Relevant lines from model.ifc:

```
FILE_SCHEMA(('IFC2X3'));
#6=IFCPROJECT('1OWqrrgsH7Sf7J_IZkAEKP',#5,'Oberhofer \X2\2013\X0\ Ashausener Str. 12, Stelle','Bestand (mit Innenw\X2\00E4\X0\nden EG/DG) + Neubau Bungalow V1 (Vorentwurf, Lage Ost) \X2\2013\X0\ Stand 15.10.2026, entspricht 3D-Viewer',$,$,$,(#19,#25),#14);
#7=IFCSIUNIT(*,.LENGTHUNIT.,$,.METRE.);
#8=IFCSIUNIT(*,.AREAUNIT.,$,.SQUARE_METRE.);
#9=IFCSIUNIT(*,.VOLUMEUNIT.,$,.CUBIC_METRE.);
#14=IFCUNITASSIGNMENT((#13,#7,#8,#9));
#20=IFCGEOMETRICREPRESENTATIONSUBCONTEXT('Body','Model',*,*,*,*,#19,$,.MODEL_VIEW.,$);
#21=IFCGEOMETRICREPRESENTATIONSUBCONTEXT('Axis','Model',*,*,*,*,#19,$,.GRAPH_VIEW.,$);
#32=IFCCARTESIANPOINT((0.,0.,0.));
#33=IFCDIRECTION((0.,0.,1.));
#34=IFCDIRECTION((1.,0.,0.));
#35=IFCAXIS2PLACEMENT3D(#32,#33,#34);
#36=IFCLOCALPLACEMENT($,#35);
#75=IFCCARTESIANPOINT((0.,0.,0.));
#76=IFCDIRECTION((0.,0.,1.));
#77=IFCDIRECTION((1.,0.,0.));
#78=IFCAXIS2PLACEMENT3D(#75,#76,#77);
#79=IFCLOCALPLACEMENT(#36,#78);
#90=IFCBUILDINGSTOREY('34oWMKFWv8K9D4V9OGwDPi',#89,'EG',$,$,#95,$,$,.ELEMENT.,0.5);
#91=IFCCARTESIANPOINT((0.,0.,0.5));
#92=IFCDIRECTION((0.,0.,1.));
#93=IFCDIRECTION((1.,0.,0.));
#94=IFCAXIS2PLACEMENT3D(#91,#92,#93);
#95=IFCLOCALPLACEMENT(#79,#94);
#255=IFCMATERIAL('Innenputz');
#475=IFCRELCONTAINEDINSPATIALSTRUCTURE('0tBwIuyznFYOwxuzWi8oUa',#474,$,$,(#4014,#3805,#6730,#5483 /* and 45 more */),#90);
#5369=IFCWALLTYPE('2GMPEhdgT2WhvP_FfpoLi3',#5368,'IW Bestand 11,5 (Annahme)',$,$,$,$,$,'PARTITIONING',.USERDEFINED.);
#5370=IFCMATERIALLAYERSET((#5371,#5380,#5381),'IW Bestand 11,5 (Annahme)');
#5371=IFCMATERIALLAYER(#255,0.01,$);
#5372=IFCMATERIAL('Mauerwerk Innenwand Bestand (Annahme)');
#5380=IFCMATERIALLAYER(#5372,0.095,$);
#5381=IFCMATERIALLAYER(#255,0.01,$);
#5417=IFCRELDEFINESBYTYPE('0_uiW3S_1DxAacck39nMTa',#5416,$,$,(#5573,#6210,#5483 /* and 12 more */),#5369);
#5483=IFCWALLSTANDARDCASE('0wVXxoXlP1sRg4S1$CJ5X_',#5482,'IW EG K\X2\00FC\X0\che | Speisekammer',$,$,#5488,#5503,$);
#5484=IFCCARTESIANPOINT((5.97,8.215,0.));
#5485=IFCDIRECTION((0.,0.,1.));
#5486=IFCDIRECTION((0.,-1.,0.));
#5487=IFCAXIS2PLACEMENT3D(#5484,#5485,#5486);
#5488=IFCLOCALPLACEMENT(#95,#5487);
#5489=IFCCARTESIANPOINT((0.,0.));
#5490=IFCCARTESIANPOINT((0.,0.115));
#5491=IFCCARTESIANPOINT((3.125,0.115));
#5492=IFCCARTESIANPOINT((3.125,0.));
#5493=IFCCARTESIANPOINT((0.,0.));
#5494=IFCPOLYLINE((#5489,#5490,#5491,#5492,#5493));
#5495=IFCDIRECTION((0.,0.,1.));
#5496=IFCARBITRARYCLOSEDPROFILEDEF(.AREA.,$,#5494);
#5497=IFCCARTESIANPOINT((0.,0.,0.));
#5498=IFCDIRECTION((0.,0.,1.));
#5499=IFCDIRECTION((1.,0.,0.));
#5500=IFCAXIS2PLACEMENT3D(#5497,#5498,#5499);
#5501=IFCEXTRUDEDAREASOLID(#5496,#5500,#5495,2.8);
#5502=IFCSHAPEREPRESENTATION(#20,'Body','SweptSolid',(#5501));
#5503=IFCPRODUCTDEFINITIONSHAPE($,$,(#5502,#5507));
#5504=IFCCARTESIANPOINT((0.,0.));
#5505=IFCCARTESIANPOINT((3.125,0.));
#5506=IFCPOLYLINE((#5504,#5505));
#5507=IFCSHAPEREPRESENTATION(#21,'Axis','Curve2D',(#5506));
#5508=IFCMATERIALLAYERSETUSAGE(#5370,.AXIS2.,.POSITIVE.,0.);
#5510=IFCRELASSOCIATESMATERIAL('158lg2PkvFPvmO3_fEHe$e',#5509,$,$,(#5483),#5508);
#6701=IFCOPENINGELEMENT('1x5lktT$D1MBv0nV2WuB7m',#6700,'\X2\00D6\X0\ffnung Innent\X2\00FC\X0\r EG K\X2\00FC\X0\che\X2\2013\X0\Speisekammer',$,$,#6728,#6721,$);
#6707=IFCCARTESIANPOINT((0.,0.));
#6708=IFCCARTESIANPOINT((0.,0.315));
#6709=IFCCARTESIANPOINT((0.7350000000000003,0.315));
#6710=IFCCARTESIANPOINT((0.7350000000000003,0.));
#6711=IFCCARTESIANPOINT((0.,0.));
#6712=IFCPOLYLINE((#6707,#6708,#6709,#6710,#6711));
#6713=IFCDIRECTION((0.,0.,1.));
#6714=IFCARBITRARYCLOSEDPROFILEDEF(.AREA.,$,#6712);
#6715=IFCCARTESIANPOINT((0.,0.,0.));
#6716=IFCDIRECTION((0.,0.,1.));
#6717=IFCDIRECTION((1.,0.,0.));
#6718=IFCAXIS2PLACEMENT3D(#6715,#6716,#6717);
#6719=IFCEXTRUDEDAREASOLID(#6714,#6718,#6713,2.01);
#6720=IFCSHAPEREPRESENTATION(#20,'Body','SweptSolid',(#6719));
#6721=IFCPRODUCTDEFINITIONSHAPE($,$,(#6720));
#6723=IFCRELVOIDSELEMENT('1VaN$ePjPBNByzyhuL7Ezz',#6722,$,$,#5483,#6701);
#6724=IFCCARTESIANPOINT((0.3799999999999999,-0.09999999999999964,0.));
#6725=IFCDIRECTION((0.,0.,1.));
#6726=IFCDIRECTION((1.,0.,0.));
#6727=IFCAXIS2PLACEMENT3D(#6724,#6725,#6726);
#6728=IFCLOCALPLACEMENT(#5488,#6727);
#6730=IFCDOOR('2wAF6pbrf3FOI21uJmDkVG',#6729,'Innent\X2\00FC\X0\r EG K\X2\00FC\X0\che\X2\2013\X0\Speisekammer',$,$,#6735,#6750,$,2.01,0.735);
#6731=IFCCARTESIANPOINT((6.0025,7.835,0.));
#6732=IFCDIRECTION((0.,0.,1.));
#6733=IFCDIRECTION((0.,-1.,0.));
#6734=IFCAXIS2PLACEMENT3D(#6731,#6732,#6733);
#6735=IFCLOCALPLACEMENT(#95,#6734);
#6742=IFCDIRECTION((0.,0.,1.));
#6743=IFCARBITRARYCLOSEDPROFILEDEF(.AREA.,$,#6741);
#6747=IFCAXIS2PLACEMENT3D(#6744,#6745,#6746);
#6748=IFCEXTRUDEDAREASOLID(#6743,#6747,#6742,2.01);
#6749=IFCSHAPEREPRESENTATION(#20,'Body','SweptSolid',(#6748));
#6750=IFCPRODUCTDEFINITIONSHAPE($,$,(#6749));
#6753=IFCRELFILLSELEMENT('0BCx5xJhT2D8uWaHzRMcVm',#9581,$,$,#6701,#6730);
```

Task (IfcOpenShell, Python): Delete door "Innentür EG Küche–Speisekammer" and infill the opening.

```python
import ifcopenshell
import ifcopenshell.api.feature
import ifcopenshell.api.root
import ifcopenshell.geom
import ifcopenshell.util.shape

model = ifcopenshell.open("model.ifc")
settings = ifcopenshell.geom.settings()


def volume(element):
    """Net volume in cubic metres, openings subtracted."""
    shape = ifcopenshell.geom.create_shape(settings, element)
    return ifcopenshell.util.shape.get_volume(shape.geometry)


door = model.by_id(6730)
opening = door.FillsVoids[0].RelatingOpeningElement
wall = opening.VoidsElements[0].RelatingBuildingElement
before = volume(wall)

ifcopenshell.api.root.remove_product(model, product=door)
ifcopenshell.api.feature.remove_feature(model, feature=opening)

after = volume(wall)

print(f"wall volume {before:.3f} -> {after:.3f} m3")

model.write("model_rev.ifc")
```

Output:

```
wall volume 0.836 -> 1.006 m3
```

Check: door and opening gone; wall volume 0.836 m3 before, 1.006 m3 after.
